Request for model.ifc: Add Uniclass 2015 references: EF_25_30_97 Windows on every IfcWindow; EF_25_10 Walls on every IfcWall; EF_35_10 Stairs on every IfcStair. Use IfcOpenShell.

First a look at what the model holds.

```python
import ifcopenshell

model = ifcopenshell.open("model.ifc")
print(model.schema)
print("classifications:", [c.Name for c in model.by_type("IfcClassification")])
for ifc_class in ("IfcDoor", "IfcRoof", "IfcStair", "IfcWall", "IfcWindow"):
    print(ifc_class, len(model.by_type(ifc_class)))
```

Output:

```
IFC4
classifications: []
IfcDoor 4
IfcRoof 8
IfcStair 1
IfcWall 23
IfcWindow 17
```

```python
import ifcopenshell
import ifcopenshell.api.classification

model = ifcopenshell.open("model.ifc")

system = ifcopenshell.api.classification.add_classification(model, classification="Uniclass 2015")

codes = {
    "IfcWindow": ("EF_25_30_97", "Windows"),
    "IfcWall": ("EF_25_10", "Walls"),
    "IfcStair": ("EF_35_10", "Stairs"),
}
for ifc_class, (code, name) in codes.items():
    products = model.by_type(ifc_class)
    ifcopenshell.api.classification.add_reference(
        model, products=products, classification=system, identification=code, name=name
    )
    print(code, len(products))

model.write("model_rev.ifc")
```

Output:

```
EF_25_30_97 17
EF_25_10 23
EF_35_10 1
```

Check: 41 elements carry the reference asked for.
